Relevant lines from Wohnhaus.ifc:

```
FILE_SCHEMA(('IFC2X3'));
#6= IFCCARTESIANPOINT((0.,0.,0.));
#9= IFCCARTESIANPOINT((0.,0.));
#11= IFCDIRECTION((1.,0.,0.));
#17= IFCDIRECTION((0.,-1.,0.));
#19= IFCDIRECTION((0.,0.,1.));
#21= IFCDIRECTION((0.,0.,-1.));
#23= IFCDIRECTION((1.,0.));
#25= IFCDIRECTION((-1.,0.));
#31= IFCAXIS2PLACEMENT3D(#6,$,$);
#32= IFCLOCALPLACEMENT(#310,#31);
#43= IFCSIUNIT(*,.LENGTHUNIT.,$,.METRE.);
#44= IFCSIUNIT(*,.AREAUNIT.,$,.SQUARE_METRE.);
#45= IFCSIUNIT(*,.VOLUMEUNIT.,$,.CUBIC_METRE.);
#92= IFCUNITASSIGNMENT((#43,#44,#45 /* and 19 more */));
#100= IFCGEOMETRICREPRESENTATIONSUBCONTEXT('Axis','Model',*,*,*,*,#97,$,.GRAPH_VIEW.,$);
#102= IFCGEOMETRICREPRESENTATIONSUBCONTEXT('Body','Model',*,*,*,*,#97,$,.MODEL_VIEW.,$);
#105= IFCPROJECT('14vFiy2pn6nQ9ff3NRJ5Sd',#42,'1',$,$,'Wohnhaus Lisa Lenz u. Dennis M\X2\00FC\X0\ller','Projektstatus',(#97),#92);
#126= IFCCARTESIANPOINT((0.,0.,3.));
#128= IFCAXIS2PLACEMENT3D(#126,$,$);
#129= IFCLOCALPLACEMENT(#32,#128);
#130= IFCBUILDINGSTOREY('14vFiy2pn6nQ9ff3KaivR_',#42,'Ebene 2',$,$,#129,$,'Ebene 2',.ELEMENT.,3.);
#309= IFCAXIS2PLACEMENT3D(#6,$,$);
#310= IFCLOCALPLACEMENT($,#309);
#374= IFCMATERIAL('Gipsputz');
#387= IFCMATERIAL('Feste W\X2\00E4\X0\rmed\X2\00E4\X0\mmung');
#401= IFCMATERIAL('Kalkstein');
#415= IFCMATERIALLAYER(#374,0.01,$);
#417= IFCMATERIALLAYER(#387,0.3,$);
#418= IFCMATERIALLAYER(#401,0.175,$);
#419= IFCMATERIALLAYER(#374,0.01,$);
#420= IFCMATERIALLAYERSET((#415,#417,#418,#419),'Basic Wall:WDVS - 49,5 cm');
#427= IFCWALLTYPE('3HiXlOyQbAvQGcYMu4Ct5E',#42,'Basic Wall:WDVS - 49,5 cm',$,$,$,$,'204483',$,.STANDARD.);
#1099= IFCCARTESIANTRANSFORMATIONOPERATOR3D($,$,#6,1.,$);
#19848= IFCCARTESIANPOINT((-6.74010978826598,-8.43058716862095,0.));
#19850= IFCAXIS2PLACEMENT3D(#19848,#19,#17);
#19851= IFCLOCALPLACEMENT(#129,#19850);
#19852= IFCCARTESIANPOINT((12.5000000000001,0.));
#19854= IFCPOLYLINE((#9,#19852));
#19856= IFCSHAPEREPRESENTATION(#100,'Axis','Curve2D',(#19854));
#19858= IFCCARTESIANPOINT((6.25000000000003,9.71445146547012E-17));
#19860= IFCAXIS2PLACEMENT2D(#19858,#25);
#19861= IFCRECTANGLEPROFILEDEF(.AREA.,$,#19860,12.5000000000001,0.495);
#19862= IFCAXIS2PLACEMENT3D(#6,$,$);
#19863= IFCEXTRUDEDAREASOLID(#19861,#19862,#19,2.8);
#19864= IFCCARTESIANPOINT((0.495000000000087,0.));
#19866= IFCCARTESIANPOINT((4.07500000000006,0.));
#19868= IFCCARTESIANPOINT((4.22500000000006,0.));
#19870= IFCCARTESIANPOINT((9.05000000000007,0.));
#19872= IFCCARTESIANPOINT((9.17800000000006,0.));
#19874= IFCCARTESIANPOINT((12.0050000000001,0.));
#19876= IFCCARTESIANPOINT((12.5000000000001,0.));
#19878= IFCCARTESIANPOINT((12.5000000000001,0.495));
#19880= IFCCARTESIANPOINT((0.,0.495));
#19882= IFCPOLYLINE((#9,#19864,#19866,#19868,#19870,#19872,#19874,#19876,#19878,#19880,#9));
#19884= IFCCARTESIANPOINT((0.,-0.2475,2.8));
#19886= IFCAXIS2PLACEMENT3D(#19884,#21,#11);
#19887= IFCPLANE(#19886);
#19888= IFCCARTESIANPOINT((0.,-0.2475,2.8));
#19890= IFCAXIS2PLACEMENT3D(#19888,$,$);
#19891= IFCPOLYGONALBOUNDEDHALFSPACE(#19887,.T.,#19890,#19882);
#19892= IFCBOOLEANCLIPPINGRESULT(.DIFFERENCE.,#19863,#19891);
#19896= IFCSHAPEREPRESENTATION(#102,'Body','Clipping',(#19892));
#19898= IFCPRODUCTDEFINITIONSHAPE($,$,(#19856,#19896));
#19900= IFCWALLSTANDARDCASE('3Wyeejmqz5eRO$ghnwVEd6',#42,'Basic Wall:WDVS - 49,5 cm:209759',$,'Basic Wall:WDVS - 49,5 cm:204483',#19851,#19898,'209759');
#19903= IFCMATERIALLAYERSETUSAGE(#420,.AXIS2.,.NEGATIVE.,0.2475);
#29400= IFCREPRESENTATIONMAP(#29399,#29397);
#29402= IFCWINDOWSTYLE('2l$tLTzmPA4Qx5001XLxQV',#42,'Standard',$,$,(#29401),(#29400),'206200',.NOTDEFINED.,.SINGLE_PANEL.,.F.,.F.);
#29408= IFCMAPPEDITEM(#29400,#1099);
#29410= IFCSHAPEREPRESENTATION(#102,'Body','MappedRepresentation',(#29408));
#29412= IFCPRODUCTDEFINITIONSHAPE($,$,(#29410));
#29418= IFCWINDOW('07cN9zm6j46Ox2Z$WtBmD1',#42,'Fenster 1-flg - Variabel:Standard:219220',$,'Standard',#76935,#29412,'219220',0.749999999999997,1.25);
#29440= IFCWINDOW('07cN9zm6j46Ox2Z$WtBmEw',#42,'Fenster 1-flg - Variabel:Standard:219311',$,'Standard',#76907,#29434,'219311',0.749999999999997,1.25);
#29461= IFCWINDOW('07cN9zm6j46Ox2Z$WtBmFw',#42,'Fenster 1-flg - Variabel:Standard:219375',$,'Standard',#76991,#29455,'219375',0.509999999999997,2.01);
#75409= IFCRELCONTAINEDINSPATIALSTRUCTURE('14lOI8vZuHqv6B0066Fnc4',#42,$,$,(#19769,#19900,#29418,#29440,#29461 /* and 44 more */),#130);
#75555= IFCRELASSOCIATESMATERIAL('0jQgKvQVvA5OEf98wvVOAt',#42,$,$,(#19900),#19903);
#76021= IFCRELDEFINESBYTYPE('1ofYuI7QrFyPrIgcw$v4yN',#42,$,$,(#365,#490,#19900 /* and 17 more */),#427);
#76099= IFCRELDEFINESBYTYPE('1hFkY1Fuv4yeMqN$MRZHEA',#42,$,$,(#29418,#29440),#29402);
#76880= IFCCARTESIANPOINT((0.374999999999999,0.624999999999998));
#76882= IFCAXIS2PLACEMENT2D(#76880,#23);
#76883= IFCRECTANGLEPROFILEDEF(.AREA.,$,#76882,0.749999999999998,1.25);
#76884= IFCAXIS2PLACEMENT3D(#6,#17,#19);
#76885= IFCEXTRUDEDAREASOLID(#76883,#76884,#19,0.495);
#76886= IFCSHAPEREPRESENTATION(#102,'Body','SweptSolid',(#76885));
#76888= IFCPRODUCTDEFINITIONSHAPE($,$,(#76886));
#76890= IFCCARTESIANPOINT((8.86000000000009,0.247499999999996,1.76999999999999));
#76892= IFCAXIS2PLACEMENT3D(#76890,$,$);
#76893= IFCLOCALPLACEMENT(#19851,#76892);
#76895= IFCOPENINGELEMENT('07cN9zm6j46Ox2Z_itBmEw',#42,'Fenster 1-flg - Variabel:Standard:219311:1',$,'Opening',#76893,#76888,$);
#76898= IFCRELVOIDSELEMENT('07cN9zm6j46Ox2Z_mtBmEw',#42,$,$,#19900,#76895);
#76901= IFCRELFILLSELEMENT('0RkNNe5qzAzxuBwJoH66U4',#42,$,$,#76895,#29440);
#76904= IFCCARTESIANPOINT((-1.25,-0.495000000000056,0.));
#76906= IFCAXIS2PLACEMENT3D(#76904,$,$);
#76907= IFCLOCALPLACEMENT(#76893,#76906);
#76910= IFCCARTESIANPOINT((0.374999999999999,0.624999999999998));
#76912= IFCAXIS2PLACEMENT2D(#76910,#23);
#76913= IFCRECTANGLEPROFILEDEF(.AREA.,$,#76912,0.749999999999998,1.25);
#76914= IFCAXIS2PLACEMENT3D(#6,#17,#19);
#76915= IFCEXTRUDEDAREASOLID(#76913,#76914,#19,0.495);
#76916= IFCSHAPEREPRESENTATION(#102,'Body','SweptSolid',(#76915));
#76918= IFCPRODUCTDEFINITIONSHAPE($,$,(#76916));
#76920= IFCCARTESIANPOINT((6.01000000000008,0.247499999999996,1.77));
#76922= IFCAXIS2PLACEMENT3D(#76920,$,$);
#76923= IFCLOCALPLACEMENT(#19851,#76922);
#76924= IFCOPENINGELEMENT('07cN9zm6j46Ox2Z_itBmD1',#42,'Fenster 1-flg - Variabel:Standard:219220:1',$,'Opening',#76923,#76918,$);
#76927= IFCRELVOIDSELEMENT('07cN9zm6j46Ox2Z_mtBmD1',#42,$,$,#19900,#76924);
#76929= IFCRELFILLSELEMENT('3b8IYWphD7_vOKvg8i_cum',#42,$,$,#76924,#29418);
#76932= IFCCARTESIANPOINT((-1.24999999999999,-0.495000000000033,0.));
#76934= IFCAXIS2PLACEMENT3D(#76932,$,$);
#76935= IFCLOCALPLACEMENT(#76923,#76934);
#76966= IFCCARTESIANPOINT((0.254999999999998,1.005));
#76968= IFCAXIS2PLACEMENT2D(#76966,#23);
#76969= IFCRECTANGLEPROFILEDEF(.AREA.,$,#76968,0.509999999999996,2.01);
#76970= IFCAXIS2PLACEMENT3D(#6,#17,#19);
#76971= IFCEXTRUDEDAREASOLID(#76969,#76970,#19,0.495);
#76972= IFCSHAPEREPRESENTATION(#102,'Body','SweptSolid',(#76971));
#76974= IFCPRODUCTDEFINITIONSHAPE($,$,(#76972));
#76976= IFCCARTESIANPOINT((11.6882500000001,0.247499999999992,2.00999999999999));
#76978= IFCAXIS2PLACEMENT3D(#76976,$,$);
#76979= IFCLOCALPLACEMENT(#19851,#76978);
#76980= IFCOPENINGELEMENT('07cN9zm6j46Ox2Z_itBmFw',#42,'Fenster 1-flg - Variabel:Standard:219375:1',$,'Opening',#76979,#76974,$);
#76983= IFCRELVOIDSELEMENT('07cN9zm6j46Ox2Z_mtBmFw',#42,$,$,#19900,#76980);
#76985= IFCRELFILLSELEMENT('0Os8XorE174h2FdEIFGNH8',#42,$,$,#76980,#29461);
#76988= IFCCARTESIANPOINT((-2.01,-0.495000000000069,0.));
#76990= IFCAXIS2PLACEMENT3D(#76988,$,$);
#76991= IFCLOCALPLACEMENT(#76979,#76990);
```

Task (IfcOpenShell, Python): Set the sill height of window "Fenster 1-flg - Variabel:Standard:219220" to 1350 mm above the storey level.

```python
import numpy as np
import ifcopenshell
import ifcopenshell.api.geometry
import ifcopenshell.geom
import ifcopenshell.util.element
import ifcopenshell.util.placement
import ifcopenshell.util.shape
import ifcopenshell.util.unit

model = ifcopenshell.open("Wohnhaus.ifc")
unit_scale = ifcopenshell.util.unit.calculate_unit_scale(model)

window = model.by_id(29418)
opening = window.FillsVoids[0].RelatingOpeningElement
storey = ifcopenshell.util.element.get_container(window, ifc_class="IfcBuildingStorey")
level = ifcopenshell.util.placement.get_local_placement(storey.ObjectPlacement)[2, 3]

# The opening's origin need not be at the sill, so measure its lowest point.
shape = ifcopenshell.geom.create_shape(ifcopenshell.geom.settings(), opening)
bottom = ifcopenshell.util.shape.get_shape_bottom_elevation(shape, shape.geometry) / unit_scale
dz = level + 1.35 / unit_scale - bottom

shift = np.array([0.0, 0.0, dz])
# The window is placed relative to its opening, so it follows when the opening moves.
matrix = ifcopenshell.util.placement.get_local_placement(opening.ObjectPlacement)
matrix[:3, 3] += shift
ifcopenshell.api.geometry.edit_object_placement(
    model, product=opening, matrix=matrix, is_si=False, should_transform_children=True
)

print(f"moved by {dz * unit_scale:+.3f} m")

model.write("Wohnhaus_v2.ifc")
```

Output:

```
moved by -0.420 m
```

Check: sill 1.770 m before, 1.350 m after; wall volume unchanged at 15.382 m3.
